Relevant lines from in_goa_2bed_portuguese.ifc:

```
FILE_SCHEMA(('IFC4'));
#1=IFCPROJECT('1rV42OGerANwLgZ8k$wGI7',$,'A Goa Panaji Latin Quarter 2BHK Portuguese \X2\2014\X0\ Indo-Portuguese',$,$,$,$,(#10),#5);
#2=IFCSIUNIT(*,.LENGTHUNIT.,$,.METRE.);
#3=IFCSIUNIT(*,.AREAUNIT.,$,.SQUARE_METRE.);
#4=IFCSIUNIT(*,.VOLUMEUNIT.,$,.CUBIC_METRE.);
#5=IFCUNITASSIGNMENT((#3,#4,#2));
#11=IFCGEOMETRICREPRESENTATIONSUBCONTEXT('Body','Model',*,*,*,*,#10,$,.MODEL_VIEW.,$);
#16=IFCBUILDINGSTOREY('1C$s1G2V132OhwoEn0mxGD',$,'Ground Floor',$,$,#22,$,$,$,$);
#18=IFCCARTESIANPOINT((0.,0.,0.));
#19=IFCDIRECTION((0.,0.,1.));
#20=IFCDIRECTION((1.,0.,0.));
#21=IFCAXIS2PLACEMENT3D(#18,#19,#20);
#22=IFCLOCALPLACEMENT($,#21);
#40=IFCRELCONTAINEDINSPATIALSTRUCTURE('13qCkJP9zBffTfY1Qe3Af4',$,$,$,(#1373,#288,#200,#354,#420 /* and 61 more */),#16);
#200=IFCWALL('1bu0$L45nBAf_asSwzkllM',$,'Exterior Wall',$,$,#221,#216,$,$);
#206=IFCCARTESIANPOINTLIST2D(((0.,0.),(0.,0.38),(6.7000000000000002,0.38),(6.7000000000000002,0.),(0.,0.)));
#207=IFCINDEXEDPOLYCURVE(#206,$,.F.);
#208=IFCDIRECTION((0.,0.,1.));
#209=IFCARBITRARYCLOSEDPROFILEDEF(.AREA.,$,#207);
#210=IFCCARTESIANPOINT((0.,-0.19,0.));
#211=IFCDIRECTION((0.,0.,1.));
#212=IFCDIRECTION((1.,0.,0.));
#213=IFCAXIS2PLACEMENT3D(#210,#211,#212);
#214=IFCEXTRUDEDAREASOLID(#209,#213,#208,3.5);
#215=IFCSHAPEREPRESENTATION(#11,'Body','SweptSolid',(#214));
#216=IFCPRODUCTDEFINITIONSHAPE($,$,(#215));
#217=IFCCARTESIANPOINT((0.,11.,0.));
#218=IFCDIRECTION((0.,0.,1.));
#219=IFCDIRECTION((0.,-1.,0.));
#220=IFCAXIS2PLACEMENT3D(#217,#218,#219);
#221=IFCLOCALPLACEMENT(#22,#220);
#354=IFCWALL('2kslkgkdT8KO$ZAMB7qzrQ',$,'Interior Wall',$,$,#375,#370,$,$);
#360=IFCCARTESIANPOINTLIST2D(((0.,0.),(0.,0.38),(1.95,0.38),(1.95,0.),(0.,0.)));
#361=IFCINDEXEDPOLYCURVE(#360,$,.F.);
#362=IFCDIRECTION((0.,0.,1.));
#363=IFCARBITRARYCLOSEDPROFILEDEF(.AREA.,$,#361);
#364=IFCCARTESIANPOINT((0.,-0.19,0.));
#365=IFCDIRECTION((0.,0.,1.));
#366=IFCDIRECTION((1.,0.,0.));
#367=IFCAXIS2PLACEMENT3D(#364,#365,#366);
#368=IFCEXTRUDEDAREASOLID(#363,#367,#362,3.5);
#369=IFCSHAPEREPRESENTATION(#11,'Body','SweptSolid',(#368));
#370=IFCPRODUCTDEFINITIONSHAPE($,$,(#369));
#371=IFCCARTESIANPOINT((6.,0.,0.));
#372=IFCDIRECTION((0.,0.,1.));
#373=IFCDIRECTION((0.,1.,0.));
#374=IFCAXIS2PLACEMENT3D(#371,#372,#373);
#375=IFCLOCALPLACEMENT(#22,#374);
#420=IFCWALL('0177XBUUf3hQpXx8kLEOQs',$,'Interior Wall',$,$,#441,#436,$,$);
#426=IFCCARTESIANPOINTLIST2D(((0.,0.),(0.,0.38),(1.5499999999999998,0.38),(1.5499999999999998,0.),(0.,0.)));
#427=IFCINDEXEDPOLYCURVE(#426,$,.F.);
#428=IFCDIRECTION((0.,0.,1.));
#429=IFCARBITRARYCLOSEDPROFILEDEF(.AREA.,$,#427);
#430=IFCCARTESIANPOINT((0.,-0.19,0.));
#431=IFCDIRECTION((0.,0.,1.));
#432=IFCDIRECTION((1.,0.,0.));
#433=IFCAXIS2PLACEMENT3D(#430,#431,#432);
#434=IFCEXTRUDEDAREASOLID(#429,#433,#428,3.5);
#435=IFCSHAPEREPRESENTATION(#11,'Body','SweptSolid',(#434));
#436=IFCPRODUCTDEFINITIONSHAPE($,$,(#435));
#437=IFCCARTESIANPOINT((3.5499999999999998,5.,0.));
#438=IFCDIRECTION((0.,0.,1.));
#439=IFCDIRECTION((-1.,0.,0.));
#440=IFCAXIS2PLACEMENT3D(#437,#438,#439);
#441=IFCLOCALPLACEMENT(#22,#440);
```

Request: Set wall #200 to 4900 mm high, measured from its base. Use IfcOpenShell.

```python
import ifcopenshell
import ifcopenshell.geom
import ifcopenshell.util.representation
import ifcopenshell.util.shape

model = ifcopenshell.open("in_goa_2bed_portuguese.ifc")
settings = ifcopenshell.geom.settings()


def volume(element):
    """Net volume in cubic metres, openings subtracted."""
    shape = ifcopenshell.geom.create_shape(settings, element)
    return ifcopenshell.util.shape.get_volume(shape.geometry)


wall = model.by_guid("1bu0$L45nBAf_asSwzkllM")
before = volume(wall)

body = ifcopenshell.util.representation.get_representation(wall, "Model", "Body")
solid = body.Items[0]
old_height = solid.Depth
solid.Depth = 4.9
after = volume(wall)

print(f"height {old_height:g} -> {solid.Depth:g}, volume {before:.3f} -> {after:.3f} m3")

model.write("in_goa_2bed_portuguese-out.ifc")
```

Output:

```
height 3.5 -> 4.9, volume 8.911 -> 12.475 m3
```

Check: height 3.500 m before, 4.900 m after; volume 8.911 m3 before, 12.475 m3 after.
